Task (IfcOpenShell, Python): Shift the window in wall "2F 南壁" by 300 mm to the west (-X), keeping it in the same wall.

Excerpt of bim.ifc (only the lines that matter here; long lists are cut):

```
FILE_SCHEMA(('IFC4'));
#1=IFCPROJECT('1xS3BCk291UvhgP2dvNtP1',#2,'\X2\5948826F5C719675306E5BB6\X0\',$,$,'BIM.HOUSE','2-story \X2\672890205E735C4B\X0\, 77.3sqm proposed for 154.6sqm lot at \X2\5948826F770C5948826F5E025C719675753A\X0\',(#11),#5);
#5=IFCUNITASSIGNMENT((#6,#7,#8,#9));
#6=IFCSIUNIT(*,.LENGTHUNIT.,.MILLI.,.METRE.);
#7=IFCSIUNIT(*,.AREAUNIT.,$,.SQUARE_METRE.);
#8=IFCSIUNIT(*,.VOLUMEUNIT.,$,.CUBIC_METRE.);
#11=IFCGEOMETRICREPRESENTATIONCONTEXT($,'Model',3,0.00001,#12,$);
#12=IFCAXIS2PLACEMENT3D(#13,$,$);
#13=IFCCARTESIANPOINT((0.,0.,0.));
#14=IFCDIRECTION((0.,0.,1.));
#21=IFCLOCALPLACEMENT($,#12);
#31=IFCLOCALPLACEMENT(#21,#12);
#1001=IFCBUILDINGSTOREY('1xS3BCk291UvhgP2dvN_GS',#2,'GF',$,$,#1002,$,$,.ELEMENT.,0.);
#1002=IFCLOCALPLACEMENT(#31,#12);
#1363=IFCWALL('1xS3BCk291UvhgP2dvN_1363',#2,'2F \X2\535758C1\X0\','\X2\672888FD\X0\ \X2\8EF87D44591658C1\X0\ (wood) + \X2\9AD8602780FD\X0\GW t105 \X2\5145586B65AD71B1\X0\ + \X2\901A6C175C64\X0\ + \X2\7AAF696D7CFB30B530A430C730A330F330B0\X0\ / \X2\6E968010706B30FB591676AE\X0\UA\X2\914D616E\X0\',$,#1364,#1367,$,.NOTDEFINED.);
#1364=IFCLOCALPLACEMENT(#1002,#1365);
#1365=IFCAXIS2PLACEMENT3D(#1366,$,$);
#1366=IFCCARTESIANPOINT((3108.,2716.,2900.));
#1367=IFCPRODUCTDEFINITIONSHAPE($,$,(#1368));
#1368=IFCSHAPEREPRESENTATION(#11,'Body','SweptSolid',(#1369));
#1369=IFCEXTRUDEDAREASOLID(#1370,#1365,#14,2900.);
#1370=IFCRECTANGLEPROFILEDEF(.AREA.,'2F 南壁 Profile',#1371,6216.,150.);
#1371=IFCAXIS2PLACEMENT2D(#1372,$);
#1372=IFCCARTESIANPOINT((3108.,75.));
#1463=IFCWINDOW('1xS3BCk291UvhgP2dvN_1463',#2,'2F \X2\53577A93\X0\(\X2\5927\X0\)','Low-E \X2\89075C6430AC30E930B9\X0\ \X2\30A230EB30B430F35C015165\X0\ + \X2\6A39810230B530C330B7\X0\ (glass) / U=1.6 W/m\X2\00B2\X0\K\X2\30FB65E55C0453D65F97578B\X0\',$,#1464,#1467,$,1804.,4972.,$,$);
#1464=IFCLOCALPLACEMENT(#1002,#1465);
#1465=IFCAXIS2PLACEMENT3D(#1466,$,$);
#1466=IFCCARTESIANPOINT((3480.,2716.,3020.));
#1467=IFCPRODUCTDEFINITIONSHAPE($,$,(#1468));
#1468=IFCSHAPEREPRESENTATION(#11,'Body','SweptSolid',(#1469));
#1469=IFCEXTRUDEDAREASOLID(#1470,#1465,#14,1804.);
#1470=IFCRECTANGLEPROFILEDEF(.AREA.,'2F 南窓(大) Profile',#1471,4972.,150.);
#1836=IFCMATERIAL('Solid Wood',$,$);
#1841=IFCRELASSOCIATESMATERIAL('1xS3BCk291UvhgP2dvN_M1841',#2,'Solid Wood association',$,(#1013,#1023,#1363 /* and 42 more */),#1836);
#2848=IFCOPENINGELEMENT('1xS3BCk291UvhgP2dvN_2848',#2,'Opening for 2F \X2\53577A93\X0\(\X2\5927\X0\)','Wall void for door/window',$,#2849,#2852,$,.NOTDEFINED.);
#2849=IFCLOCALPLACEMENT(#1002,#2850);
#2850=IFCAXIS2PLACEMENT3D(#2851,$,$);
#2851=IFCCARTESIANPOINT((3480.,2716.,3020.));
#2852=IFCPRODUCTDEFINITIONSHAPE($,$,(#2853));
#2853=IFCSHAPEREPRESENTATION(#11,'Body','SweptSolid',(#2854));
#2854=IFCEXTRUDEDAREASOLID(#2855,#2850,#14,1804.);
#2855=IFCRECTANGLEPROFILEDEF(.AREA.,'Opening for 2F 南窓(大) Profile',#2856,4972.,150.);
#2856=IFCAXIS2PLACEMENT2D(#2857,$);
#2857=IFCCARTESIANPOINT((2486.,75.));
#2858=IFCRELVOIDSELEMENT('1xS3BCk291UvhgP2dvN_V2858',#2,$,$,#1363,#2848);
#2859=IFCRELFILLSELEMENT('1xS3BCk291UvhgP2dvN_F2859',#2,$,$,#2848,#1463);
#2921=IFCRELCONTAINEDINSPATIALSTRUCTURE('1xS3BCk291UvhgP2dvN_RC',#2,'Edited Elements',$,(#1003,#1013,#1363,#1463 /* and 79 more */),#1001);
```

```python
import ifcopenshell
import ifcopenshell.api.geometry
import ifcopenshell.util.placement
import ifcopenshell.util.unit

model = ifcopenshell.open("bim.ifc")
unit_scale = ifcopenshell.util.unit.calculate_unit_scale(model)

window = model.by_id(1463)
opening = window.FillsVoids[0].RelatingOpeningElement
wall = opening.VoidsElements[0].RelatingBuildingElement

wall_matrix = ifcopenshell.util.placement.get_local_placement(wall.ObjectPlacement)
shift = wall_matrix[:3, 0] * -0.3 / unit_scale
before = ifcopenshell.util.placement.get_local_placement(window.ObjectPlacement)[:3, 3].copy()

# The window is not placed relative to its opening, so move both.
for product in (opening, window):
    matrix = ifcopenshell.util.placement.get_local_placement(product.ObjectPlacement)
    matrix[:3, 3] += shift
    ifcopenshell.api.geometry.edit_object_placement(model, product=product, matrix=matrix, is_si=False)

after = ifcopenshell.util.placement.get_local_placement(window.ObjectPlacement)[:3, 3]
print("window moved by", (after - before).round(3) + 0.0)

model.write("bim-out.ifc")
```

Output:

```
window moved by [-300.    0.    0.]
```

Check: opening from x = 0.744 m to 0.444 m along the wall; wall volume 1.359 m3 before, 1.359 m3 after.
